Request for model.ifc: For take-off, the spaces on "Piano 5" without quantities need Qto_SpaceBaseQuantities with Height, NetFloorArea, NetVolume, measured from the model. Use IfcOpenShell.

First a look at what the model holds.

```python
import ifcopenshell
import ifcopenshell.util.element
import ifcopenshell.util.unit

model = ifcopenshell.open("model.ifc")
print(model.schema)
for unit_type in ("LENGTHUNIT", "AREAUNIT", "VOLUMEUNIT"):
    print(unit_type, ifcopenshell.util.unit.calculate_unit_scale(model, unit_type))
storey = next(s for s in model.by_type("IfcBuildingStorey") if s.Name == "Piano 5")
spaces = [e for e in ifcopenshell.util.element.get_decomposition(storey) if e.is_a("IfcSpace")]
for e in sorted(spaces, key=lambda e: e.id()):
    print(e.id(), e.is_a(), e.Name, list(ifcopenshell.util.element.get_psets(e, qtos_only=True)), sep=" | ")
```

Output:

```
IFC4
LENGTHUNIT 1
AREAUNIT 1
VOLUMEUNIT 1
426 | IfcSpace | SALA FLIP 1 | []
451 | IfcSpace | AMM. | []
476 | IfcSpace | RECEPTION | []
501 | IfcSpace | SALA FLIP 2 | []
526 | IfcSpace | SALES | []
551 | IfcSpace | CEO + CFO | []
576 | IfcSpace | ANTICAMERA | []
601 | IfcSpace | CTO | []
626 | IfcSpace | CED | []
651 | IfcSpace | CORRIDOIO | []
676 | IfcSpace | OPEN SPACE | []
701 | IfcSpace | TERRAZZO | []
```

```python
import ifcopenshell
import ifcopenshell.api.pset
import ifcopenshell.geom
import ifcopenshell.util.element
import ifcopenshell.util.shape
import ifcopenshell.util.unit

model = ifcopenshell.open("model.ifc")
unit_scale = ifcopenshell.util.unit.calculate_unit_scale(model)
area_scale = ifcopenshell.util.unit.calculate_unit_scale(model, "AREAUNIT")
volume_scale = ifcopenshell.util.unit.calculate_unit_scale(model, "VOLUMEUNIT")
settings = ifcopenshell.geom.settings()

storey = next(s for s in model.by_type("IfcBuildingStorey") if s.Name == "Piano 5")
spaces = [e for e in ifcopenshell.util.element.get_decomposition(storey) if e.is_a("IfcSpace")]

for e in sorted(spaces, key=lambda e: e.id()):
    if ifcopenshell.util.element.get_psets(e, qtos_only=True, should_inherit=False):
        continue
    # Geometry comes back in metres, in the element's own axes.
    shape = ifcopenshell.geom.create_shape(settings, e)
    values = {
        "Height": ifcopenshell.util.shape.get_z(shape.geometry) / unit_scale,
        "NetFloorArea": ifcopenshell.util.shape.get_footprint_area(shape.geometry) / area_scale,
        "NetVolume": ifcopenshell.util.shape.get_volume(shape.geometry) / volume_scale,
    }
    qto = ifcopenshell.api.pset.add_qto(model, product=e, name="Qto_SpaceBaseQuantities")
    ifcopenshell.api.pset.edit_qto(model, qto=qto, properties=values)
    print(e.id(), {k: round(v, 3) for k, v in values.items()})

model.write("model_edited.ifc")
```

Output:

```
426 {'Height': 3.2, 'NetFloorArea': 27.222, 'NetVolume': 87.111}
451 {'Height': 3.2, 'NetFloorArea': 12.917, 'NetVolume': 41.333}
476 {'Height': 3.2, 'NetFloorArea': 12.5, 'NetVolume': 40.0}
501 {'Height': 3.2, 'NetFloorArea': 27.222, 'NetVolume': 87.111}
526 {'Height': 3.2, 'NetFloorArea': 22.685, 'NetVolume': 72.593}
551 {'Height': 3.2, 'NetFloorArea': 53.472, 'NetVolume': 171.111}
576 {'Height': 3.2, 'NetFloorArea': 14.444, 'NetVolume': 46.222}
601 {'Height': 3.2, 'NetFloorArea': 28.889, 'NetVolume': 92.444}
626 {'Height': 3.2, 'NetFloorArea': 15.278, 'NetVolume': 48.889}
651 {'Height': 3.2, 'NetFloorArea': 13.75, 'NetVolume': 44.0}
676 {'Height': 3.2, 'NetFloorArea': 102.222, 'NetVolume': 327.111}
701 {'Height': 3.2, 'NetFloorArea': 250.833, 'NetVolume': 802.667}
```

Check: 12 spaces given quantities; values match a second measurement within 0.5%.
